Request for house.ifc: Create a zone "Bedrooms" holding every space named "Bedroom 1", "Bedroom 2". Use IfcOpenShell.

First a look at what the model holds.

```python
import ifcopenshell

model = ifcopenshell.open("house.ifc")
print(model.schema)
seen = {}
for space in model.by_type("IfcSpace"):
    seen[space.LongName] = seen.get(space.LongName, 0) + 1
for name, count in sorted(seen.items(), key=str):
    print(count, "x", name)
print("zones:", [z.Name for z in model.by_type("IfcZone")][:20])
```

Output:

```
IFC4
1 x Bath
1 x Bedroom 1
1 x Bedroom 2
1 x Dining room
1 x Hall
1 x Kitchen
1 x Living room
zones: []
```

```python
import ifcopenshell
import ifcopenshell.api.group
import ifcopenshell.api.root

model = ifcopenshell.open("house.ifc")

names = {"Bedroom 1", "Bedroom 2"}
spaces = [s for s in model.by_type("IfcSpace") if s.LongName in names]

zone = ifcopenshell.api.root.create_entity(model, ifc_class="IfcZone", name="Bedrooms")
ifcopenshell.api.group.assign_group(model, products=spaces, group=zone)
print(len(spaces), "spaces in", zone.Name)

model.write("house_v2.ifc")
```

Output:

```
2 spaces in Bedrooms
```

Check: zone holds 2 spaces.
